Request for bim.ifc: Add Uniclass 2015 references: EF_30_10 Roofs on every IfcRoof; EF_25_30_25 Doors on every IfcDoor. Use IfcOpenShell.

First a look at what the model holds.

```python
import ifcopenshell

model = ifcopenshell.open("bim.ifc")
print(model.schema)
print("classifications:", [c.Name for c in model.by_type("IfcClassification")])
for ifc_class in ("IfcDoor", "IfcRoof", "IfcStair", "IfcWall", "IfcWindow"):
    print(ifc_class, len(model.by_type(ifc_class)))
```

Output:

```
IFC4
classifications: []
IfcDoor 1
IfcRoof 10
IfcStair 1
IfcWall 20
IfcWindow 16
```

```python
import ifcopenshell
import ifcopenshell.api.classification

model = ifcopenshell.open("bim.ifc")

system = ifcopenshell.api.classification.add_classification(model, classification="Uniclass 2015")

codes = {
    "IfcRoof": ("EF_30_10", "Roofs"),
    "IfcDoor": ("EF_25_30_25", "Doors"),
}
for ifc_class, (code, name) in codes.items():
    products = model.by_type(ifc_class)
    ifcopenshell.api.classification.add_reference(
        model, products=products, classification=system, identification=code, name=name
    )
    print(code, len(products))

model.write("bim-out.ifc")
```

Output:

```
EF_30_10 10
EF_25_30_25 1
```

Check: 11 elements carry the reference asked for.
